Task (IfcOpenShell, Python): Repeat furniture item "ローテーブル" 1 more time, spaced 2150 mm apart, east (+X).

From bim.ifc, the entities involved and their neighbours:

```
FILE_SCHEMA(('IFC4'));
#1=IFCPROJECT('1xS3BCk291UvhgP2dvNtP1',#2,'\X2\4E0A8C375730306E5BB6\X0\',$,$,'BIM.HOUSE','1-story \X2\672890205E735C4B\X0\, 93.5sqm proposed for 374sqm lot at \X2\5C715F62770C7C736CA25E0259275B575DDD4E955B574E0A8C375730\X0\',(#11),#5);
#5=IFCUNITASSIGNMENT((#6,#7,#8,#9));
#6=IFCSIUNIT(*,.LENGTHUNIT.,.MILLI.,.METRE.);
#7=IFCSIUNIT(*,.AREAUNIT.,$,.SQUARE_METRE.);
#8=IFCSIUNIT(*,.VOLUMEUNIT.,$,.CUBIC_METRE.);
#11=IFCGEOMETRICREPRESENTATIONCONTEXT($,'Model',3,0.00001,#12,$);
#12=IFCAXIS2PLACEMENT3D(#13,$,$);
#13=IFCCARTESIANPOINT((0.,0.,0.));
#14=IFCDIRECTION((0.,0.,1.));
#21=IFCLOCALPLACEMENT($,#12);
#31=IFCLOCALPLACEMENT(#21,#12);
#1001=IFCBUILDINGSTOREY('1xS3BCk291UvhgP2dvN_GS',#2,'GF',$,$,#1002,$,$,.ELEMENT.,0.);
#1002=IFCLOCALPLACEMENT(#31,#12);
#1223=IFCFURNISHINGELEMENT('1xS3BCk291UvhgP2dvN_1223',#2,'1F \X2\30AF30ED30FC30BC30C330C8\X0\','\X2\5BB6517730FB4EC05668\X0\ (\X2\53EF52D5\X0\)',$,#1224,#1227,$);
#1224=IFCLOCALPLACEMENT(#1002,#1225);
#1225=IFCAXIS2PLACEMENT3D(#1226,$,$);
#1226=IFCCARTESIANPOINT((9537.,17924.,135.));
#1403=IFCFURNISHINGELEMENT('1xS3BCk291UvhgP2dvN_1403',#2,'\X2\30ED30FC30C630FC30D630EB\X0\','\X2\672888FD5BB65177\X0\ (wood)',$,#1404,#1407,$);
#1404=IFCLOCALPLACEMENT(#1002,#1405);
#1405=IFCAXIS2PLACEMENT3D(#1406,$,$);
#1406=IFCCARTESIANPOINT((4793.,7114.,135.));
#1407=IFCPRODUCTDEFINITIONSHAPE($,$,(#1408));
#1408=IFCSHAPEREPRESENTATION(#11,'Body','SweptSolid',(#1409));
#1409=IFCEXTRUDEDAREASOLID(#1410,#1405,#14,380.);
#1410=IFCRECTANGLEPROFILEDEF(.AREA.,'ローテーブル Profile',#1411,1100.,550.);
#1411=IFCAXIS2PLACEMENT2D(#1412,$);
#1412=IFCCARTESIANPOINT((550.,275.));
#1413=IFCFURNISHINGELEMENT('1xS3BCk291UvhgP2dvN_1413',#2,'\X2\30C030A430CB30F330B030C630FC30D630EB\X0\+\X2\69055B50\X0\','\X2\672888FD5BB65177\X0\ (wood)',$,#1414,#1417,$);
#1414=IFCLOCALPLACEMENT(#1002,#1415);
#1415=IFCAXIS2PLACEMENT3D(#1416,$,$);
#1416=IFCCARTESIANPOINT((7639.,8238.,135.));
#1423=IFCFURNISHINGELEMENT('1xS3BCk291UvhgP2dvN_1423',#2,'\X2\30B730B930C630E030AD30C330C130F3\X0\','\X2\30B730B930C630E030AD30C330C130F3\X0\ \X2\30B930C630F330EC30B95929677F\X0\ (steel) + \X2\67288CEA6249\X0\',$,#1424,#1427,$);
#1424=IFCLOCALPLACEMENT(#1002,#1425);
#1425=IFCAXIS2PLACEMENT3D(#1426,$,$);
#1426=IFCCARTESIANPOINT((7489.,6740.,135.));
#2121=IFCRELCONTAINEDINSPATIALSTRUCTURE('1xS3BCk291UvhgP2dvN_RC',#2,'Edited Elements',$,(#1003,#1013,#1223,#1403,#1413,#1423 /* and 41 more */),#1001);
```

```python
import numpy as np
import ifcopenshell
import ifcopenshell.api.geometry
import ifcopenshell.api.root
import ifcopenshell.util.element
import ifcopenshell.util.placement

model = ifcopenshell.open("bim.ifc")


def reuse_history(source, copy):
    """copy_class also copies each property set's owner history, people and application; keep the originals."""
    for rel in copy.IsDefinedBy:
        if rel.is_a("IfcRelDefinesByProperties") and (history := rel.RelatingPropertyDefinition.OwnerHistory):
            rel.RelatingPropertyDefinition.OwnerHistory = source.OwnerHistory
            ifcopenshell.util.element.remove_deep2(model, history)


source = model.by_guid("1xS3BCk291UvhgP2dvN_1403")
base = ifcopenshell.util.placement.get_local_placement(source.ObjectPlacement)
step = np.array([1.0, 0.0, 0.0]) * 2150.0

for i in range(1, 2):
    copy = ifcopenshell.api.root.copy_class(model, product=source)
    copy.Representation = ifcopenshell.util.element.copy_deep(
        model, source.Representation, exclude=["IfcGeometricRepresentationContext", "IfcRepresentationMap"]
    )
    reuse_history(source, copy)
    matrix = base.copy()
    matrix[:3, 3] += i * step
    print("added at", matrix[:3, 3].round(3) + 0.0)
    ifcopenshell.api.geometry.edit_object_placement(model, product=copy, matrix=matrix, is_si=False)

model.write("bim_rev.ifc")
```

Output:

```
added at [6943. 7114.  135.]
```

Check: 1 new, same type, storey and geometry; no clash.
